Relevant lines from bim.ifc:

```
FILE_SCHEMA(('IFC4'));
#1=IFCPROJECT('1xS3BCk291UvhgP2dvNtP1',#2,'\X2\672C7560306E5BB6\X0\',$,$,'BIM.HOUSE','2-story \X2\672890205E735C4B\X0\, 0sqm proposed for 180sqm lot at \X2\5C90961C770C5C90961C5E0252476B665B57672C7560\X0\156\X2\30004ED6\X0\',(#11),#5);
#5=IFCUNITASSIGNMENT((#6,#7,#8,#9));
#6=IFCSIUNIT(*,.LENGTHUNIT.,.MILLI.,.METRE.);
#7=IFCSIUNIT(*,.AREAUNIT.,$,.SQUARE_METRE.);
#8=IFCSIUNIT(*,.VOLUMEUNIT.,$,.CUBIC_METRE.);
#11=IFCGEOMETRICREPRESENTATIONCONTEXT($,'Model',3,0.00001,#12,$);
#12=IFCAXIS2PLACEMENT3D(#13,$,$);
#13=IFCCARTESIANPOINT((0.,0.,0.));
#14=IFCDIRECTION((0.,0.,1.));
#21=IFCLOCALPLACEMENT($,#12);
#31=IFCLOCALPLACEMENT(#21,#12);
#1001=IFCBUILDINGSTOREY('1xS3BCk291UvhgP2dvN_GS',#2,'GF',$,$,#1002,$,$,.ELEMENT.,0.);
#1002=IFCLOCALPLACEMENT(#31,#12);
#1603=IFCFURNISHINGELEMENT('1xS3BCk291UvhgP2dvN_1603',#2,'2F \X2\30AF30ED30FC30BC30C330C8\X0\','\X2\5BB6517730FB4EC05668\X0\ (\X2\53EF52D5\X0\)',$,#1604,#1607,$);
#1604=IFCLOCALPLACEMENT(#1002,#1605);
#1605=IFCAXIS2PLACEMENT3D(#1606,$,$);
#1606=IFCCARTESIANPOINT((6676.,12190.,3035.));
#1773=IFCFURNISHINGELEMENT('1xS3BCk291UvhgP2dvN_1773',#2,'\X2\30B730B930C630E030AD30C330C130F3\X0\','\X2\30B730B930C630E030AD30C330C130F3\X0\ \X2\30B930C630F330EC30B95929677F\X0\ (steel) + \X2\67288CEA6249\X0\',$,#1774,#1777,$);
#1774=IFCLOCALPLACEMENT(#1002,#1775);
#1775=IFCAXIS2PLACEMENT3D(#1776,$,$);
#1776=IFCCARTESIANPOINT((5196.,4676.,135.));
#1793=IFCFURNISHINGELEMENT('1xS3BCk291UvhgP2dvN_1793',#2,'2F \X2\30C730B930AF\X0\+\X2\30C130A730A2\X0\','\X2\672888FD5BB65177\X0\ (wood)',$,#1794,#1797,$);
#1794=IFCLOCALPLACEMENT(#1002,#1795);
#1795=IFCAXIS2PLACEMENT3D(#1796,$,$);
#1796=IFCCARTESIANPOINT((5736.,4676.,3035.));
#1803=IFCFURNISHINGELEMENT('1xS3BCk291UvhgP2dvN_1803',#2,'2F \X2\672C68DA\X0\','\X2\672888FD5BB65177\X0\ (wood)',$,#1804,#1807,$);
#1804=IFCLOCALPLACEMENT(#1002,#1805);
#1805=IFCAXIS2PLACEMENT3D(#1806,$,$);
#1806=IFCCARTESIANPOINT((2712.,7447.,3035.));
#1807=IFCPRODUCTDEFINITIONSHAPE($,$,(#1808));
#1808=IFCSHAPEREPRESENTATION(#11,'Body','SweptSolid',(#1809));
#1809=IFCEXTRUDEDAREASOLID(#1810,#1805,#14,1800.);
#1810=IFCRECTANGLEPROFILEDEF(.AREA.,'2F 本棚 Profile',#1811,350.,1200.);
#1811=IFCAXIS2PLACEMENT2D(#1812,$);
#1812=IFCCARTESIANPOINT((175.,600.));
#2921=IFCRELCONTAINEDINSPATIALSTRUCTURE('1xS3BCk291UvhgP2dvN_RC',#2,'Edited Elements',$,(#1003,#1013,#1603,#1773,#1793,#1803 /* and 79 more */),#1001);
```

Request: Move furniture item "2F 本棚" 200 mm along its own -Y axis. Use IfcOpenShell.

```python
import ifcopenshell
import ifcopenshell.api.geometry
import ifcopenshell.util.placement
import ifcopenshell.util.unit

model = ifcopenshell.open("bim.ifc")
unit_scale = ifcopenshell.util.unit.calculate_unit_scale(model)

item = model.by_guid("1xS3BCk291UvhgP2dvN_1803")
matrix = ifcopenshell.util.placement.get_local_placement(item.ObjectPlacement)
matrix[:3, 3] -= matrix[:3, 1] * 0.2 / unit_scale
ifcopenshell.api.geometry.edit_object_placement(model, product=item, matrix=matrix, is_si=False)

print(ifcopenshell.util.placement.get_local_placement(item.ObjectPlacement).round(3) + 0.0)

model.write("bim_updated.ifc")
```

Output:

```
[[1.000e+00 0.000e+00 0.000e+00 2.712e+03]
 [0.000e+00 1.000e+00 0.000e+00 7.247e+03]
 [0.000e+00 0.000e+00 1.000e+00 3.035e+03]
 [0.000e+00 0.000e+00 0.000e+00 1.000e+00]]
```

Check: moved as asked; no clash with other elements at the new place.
